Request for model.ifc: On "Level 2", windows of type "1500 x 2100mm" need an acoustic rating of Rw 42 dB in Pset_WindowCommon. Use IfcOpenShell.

First a look at what the model holds.

```python
import ifcopenshell
import ifcopenshell.util.element

model = ifcopenshell.open("model.ifc")
print(model.schema)
storey = next(s for s in model.by_type("IfcBuildingStorey") if s.Name == "Level 2")
windows = [e for e in ifcopenshell.util.element.get_decomposition(storey) if e.is_a("IfcWindow")]
seen = {}
for e in windows:
    element_type = ifcopenshell.util.element.get_type(e)
    key = (element_type.Name if element_type != e and element_type else None, ifcopenshell.util.element.get_pset(e, "Pset_WindowCommon", "AcousticRating"))
    seen[key] = seen.get(key, 0) + 1
for (name, value), count in sorted(seen.items(), key=str):
    print(count, "x", name, "|", value)
```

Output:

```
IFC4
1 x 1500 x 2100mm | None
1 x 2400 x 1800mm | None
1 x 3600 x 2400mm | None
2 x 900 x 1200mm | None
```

```python
import ifcopenshell
import ifcopenshell.api.pset
import ifcopenshell.util.element

model = ifcopenshell.open("model.ifc")

storey = next(s for s in model.by_type("IfcBuildingStorey") if s.Name == "Level 2")
windows = [e for e in ifcopenshell.util.element.get_decomposition(storey) if e.is_a("IfcWindow")]

count = 0
for e in windows:
    element_type = ifcopenshell.util.element.get_type(e)
    if element_type in (None, e) or element_type.Name != "1500 x 2100mm":
        continue
    # add_pset returns the element's existing set when there is one.
    pset = ifcopenshell.api.pset.add_pset(model, product=e, name="Pset_WindowCommon")
    ifcopenshell.api.pset.edit_pset(model, pset=pset, properties={"AcousticRating": "Rw 42 dB"})
    count += 1

print(count, "windows updated")

model.write("model_v2.ifc")
```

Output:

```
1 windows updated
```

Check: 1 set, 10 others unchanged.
